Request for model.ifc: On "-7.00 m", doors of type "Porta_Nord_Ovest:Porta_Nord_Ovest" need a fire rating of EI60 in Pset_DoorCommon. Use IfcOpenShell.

First a look at what the model holds.

```python
import ifcopenshell
import ifcopenshell.util.element

model = ifcopenshell.open("model.ifc")
print(model.schema)
storey = next(s for s in model.by_type("IfcBuildingStorey") if s.Name == "-7.00 m")
doors = [e for e in ifcopenshell.util.element.get_decomposition(storey) if e.is_a("IfcDoor")]
seen = {}
for e in doors:
    element_type = ifcopenshell.util.element.get_type(e)
    key = (element_type.Name if element_type != e and element_type else None, ifcopenshell.util.element.get_pset(e, "Pset_DoorCommon", "FireRating"))
    seen[key] = seen.get(key, 0) + 1
for (name, value), count in sorted(seen.items(), key=str):
    print(count, "x", name, "|", value)
```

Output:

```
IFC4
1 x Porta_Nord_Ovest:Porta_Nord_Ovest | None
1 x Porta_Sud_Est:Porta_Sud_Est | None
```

```python
import ifcopenshell
import ifcopenshell.api.pset
import ifcopenshell.util.element

model = ifcopenshell.open("model.ifc")

storey = next(s for s in model.by_type("IfcBuildingStorey") if s.Name == "-7.00 m")
doors = [e for e in ifcopenshell.util.element.get_decomposition(storey) if e.is_a("IfcDoor")]

count = 0
for e in doors:
    element_type = ifcopenshell.util.element.get_type(e)
    if element_type in (None, e) or element_type.Name != "Porta_Nord_Ovest:Porta_Nord_Ovest":
        continue
    # add_pset returns the element's existing set when there is one.
    pset = ifcopenshell.api.pset.add_pset(model, product=e, name="Pset_DoorCommon")
    ifcopenshell.api.pset.edit_pset(model, pset=pset, properties={"FireRating": "EI60"})
    count += 1

print(count, "doors updated")

model.write("model_updated.ifc")
```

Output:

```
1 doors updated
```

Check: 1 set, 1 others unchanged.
